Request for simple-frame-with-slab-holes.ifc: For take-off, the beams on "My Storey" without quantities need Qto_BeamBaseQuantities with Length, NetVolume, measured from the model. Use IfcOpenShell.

First a look at what the model holds.

```python
import ifcopenshell
import ifcopenshell.util.element
import ifcopenshell.util.unit

model = ifcopenshell.open("simple-frame-with-slab-holes.ifc")
print(model.schema)
for unit_type in ("LENGTHUNIT", "AREAUNIT", "VOLUMEUNIT"):
    print(unit_type, ifcopenshell.util.unit.calculate_unit_scale(model, unit_type))
storey = next(s for s in model.by_type("IfcBuildingStorey") if s.Name == "My Storey")
beams = [e for e in ifcopenshell.util.element.get_decomposition(storey) if e.is_a("IfcBeam")]
for e in sorted(beams, key=lambda e: e.id()):
    print(e.id(), e.is_a(), e.Name, list(ifcopenshell.util.element.get_psets(e, qtos_only=True)), sep=" | ")
```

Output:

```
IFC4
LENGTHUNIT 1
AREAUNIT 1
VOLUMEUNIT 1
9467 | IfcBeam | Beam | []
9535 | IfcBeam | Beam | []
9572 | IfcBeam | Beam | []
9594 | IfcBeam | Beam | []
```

```python
import ifcopenshell
import ifcopenshell.api.pset
import ifcopenshell.geom
import ifcopenshell.util.element
import ifcopenshell.util.shape
import ifcopenshell.util.unit

model = ifcopenshell.open("simple-frame-with-slab-holes.ifc")
unit_scale = ifcopenshell.util.unit.calculate_unit_scale(model)
volume_scale = ifcopenshell.util.unit.calculate_unit_scale(model, "VOLUMEUNIT")
settings = ifcopenshell.geom.settings()

storey = next(s for s in model.by_type("IfcBuildingStorey") if s.Name == "My Storey")
beams = [e for e in ifcopenshell.util.element.get_decomposition(storey) if e.is_a("IfcBeam")]

for e in sorted(beams, key=lambda e: e.id()):
    if ifcopenshell.util.element.get_psets(e, qtos_only=True, should_inherit=False):
        continue
    # Geometry comes back in metres, in the element's own axes.
    shape = ifcopenshell.geom.create_shape(settings, e)
    values = {
        "Length": ifcopenshell.util.shape.get_max_xyz(shape.geometry) / unit_scale,
        "NetVolume": ifcopenshell.util.shape.get_volume(shape.geometry) / volume_scale,
    }
    qto = ifcopenshell.api.pset.add_qto(model, product=e, name="Qto_BeamBaseQuantities")
    ifcopenshell.api.pset.edit_qto(model, qto=qto, properties=values)
    print(e.id(), {k: round(v, 3) for k, v in values.items()})

model.write("simple-frame-with-slab-holes_edited.ifc")
```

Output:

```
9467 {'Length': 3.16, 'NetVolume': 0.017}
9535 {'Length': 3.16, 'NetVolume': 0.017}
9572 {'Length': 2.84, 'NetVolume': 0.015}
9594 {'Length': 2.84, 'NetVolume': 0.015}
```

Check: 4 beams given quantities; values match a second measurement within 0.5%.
